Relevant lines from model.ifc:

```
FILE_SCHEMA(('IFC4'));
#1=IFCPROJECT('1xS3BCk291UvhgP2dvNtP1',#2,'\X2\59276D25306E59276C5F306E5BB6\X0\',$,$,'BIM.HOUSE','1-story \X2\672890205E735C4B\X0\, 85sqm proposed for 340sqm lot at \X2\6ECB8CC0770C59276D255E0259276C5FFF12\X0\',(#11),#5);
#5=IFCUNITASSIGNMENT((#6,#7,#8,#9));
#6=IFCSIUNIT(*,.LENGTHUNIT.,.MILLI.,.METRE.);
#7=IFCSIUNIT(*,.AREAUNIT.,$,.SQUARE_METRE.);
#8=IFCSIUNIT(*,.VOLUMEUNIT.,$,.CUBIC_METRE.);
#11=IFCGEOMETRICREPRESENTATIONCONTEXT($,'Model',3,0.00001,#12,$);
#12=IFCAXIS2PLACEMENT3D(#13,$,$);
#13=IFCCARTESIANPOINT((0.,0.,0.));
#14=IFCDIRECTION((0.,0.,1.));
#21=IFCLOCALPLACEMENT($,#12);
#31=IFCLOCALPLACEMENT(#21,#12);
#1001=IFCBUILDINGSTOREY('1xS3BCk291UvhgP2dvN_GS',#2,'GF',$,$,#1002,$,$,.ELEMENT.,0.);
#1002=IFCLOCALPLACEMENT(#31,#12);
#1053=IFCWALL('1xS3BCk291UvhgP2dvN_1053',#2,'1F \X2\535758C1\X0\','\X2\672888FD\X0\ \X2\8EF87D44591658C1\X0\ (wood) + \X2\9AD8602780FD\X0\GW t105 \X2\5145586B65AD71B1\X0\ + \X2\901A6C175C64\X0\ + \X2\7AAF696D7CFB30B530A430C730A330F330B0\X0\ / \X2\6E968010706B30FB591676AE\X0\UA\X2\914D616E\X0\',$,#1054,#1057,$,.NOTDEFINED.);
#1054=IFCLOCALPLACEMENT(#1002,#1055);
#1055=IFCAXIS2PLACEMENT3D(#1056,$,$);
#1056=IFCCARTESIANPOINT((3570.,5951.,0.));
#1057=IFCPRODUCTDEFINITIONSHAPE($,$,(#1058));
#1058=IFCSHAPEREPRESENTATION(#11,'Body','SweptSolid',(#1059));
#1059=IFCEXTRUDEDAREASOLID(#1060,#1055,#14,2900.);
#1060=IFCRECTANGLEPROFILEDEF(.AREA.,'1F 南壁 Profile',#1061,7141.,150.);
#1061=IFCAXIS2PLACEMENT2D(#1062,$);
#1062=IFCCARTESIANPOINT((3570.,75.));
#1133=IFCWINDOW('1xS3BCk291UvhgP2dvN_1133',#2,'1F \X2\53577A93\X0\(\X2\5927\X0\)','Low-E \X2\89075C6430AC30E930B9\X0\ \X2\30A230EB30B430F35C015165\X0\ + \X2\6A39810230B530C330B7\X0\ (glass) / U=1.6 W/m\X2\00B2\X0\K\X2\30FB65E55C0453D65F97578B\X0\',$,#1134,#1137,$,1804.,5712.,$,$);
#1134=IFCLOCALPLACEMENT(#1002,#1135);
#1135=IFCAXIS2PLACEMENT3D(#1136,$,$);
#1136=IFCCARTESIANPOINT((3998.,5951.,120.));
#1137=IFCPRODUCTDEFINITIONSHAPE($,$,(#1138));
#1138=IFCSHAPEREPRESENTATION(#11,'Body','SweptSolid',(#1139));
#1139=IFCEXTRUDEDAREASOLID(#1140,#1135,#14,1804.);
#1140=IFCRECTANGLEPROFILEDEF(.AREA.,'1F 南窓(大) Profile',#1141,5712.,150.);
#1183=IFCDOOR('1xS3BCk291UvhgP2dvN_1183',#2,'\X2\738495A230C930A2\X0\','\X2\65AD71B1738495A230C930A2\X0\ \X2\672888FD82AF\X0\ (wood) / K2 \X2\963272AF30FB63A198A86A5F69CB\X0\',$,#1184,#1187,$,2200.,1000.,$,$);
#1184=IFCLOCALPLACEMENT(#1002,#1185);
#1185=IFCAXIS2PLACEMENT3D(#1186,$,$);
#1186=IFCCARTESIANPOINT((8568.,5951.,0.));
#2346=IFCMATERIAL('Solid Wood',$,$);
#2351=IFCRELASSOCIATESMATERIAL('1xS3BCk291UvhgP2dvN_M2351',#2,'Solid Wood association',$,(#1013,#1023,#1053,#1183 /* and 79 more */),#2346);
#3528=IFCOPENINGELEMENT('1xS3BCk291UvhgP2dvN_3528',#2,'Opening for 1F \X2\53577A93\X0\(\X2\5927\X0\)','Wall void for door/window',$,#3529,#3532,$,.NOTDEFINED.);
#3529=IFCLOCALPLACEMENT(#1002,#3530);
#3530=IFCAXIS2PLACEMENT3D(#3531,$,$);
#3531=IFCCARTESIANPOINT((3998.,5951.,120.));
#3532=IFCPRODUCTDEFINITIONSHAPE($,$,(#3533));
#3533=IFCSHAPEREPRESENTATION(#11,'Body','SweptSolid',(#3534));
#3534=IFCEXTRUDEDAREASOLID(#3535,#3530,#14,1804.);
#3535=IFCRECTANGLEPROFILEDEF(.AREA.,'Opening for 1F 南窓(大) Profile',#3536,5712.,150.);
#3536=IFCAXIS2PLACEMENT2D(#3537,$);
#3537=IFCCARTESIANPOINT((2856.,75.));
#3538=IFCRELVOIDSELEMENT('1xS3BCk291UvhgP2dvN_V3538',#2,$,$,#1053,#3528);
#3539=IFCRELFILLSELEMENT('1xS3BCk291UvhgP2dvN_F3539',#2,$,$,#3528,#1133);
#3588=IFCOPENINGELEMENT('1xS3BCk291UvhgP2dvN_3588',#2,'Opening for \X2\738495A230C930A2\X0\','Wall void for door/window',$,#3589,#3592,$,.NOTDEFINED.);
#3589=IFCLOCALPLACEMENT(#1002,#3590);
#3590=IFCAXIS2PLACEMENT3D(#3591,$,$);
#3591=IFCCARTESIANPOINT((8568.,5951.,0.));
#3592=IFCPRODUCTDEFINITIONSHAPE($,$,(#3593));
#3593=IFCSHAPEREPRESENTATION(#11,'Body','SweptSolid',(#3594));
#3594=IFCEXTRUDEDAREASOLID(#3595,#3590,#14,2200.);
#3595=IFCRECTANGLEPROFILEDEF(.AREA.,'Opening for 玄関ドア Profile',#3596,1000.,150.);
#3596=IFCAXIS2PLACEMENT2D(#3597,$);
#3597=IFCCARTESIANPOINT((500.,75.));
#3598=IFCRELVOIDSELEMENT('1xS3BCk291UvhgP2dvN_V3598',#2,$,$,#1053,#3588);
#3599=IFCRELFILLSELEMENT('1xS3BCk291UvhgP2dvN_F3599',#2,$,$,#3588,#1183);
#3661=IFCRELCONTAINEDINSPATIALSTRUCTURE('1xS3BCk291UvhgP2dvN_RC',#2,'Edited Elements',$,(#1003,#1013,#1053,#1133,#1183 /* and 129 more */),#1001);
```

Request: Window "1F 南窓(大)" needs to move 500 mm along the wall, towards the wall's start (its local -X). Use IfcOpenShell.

```python
import ifcopenshell
import ifcopenshell.api.geometry
import ifcopenshell.util.placement
import ifcopenshell.util.unit

model = ifcopenshell.open("model.ifc")
unit_scale = ifcopenshell.util.unit.calculate_unit_scale(model)

window = model.by_guid("1xS3BCk291UvhgP2dvN_1133")
opening = window.FillsVoids[0].RelatingOpeningElement
wall = opening.VoidsElements[0].RelatingBuildingElement

wall_matrix = ifcopenshell.util.placement.get_local_placement(wall.ObjectPlacement)
shift = wall_matrix[:3, 0] * -0.5 / unit_scale
before = ifcopenshell.util.placement.get_local_placement(window.ObjectPlacement)[:3, 3].copy()

# The window is not placed relative to its opening, so move both.
for product in (opening, window):
    matrix = ifcopenshell.util.placement.get_local_placement(product.ObjectPlacement)
    matrix[:3, 3] += shift
    ifcopenshell.api.geometry.edit_object_placement(model, product=product, matrix=matrix, is_si=False)

after = ifcopenshell.util.placement.get_local_placement(window.ObjectPlacement)[:3, 3]
print("window moved by", (after - before).round(3) + 0.0)

model.write("model_v2.ifc")
```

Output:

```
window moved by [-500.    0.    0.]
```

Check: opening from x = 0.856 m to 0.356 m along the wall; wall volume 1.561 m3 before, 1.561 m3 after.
